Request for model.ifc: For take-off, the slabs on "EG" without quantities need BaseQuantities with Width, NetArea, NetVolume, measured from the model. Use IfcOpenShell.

First a look at what the model holds.

```python
import ifcopenshell
import ifcopenshell.util.element
import ifcopenshell.util.unit

model = ifcopenshell.open("model.ifc")
print(model.schema)
for unit_type in ("LENGTHUNIT", "AREAUNIT", "VOLUMEUNIT"):
    print(unit_type, ifcopenshell.util.unit.calculate_unit_scale(model, unit_type))
storey = next(s for s in model.by_type("IfcBuildingStorey") if s.Name == "EG")
slabs = [e for e in ifcopenshell.util.element.get_decomposition(storey) if e.is_a("IfcSlab")]
for e in sorted(slabs, key=lambda e: e.id()):
    print(e.id(), e.is_a(), e.Name, list(ifcopenshell.util.element.get_psets(e, qtos_only=True)), sep=" | ")
```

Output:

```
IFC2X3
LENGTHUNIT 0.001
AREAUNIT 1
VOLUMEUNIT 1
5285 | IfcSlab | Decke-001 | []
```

```python
import ifcopenshell
import ifcopenshell.api.pset
import ifcopenshell.geom
import ifcopenshell.util.element
import ifcopenshell.util.shape
import ifcopenshell.util.unit

model = ifcopenshell.open("model.ifc")
unit_scale = ifcopenshell.util.unit.calculate_unit_scale(model)
area_scale = ifcopenshell.util.unit.calculate_unit_scale(model, "AREAUNIT")
volume_scale = ifcopenshell.util.unit.calculate_unit_scale(model, "VOLUMEUNIT")
settings = ifcopenshell.geom.settings()

storey = next(s for s in model.by_type("IfcBuildingStorey") if s.Name == "EG")
slabs = [e for e in ifcopenshell.util.element.get_decomposition(storey) if e.is_a("IfcSlab")]

for e in sorted(slabs, key=lambda e: e.id()):
    if ifcopenshell.util.element.get_psets(e, qtos_only=True, should_inherit=False):
        continue
    # Geometry comes back in metres, in the element's own axes.
    shape = ifcopenshell.geom.create_shape(settings, e)
    values = {
        "Width": ifcopenshell.util.shape.get_z(shape.geometry) / unit_scale,
        "NetArea": ifcopenshell.util.shape.get_footprint_area(shape.geometry) / area_scale,
        "NetVolume": ifcopenshell.util.shape.get_volume(shape.geometry) / volume_scale,
    }
    qto = ifcopenshell.api.pset.add_qto(model, product=e, name="BaseQuantities")
    ifcopenshell.api.pset.edit_qto(model, qto=qto, properties=values)
    print(e.id(), {k: round(v, 3) for k, v in values.items()})

model.write("model_rev.ifc")
```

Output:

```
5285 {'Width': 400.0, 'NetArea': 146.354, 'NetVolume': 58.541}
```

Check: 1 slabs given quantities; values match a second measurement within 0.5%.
